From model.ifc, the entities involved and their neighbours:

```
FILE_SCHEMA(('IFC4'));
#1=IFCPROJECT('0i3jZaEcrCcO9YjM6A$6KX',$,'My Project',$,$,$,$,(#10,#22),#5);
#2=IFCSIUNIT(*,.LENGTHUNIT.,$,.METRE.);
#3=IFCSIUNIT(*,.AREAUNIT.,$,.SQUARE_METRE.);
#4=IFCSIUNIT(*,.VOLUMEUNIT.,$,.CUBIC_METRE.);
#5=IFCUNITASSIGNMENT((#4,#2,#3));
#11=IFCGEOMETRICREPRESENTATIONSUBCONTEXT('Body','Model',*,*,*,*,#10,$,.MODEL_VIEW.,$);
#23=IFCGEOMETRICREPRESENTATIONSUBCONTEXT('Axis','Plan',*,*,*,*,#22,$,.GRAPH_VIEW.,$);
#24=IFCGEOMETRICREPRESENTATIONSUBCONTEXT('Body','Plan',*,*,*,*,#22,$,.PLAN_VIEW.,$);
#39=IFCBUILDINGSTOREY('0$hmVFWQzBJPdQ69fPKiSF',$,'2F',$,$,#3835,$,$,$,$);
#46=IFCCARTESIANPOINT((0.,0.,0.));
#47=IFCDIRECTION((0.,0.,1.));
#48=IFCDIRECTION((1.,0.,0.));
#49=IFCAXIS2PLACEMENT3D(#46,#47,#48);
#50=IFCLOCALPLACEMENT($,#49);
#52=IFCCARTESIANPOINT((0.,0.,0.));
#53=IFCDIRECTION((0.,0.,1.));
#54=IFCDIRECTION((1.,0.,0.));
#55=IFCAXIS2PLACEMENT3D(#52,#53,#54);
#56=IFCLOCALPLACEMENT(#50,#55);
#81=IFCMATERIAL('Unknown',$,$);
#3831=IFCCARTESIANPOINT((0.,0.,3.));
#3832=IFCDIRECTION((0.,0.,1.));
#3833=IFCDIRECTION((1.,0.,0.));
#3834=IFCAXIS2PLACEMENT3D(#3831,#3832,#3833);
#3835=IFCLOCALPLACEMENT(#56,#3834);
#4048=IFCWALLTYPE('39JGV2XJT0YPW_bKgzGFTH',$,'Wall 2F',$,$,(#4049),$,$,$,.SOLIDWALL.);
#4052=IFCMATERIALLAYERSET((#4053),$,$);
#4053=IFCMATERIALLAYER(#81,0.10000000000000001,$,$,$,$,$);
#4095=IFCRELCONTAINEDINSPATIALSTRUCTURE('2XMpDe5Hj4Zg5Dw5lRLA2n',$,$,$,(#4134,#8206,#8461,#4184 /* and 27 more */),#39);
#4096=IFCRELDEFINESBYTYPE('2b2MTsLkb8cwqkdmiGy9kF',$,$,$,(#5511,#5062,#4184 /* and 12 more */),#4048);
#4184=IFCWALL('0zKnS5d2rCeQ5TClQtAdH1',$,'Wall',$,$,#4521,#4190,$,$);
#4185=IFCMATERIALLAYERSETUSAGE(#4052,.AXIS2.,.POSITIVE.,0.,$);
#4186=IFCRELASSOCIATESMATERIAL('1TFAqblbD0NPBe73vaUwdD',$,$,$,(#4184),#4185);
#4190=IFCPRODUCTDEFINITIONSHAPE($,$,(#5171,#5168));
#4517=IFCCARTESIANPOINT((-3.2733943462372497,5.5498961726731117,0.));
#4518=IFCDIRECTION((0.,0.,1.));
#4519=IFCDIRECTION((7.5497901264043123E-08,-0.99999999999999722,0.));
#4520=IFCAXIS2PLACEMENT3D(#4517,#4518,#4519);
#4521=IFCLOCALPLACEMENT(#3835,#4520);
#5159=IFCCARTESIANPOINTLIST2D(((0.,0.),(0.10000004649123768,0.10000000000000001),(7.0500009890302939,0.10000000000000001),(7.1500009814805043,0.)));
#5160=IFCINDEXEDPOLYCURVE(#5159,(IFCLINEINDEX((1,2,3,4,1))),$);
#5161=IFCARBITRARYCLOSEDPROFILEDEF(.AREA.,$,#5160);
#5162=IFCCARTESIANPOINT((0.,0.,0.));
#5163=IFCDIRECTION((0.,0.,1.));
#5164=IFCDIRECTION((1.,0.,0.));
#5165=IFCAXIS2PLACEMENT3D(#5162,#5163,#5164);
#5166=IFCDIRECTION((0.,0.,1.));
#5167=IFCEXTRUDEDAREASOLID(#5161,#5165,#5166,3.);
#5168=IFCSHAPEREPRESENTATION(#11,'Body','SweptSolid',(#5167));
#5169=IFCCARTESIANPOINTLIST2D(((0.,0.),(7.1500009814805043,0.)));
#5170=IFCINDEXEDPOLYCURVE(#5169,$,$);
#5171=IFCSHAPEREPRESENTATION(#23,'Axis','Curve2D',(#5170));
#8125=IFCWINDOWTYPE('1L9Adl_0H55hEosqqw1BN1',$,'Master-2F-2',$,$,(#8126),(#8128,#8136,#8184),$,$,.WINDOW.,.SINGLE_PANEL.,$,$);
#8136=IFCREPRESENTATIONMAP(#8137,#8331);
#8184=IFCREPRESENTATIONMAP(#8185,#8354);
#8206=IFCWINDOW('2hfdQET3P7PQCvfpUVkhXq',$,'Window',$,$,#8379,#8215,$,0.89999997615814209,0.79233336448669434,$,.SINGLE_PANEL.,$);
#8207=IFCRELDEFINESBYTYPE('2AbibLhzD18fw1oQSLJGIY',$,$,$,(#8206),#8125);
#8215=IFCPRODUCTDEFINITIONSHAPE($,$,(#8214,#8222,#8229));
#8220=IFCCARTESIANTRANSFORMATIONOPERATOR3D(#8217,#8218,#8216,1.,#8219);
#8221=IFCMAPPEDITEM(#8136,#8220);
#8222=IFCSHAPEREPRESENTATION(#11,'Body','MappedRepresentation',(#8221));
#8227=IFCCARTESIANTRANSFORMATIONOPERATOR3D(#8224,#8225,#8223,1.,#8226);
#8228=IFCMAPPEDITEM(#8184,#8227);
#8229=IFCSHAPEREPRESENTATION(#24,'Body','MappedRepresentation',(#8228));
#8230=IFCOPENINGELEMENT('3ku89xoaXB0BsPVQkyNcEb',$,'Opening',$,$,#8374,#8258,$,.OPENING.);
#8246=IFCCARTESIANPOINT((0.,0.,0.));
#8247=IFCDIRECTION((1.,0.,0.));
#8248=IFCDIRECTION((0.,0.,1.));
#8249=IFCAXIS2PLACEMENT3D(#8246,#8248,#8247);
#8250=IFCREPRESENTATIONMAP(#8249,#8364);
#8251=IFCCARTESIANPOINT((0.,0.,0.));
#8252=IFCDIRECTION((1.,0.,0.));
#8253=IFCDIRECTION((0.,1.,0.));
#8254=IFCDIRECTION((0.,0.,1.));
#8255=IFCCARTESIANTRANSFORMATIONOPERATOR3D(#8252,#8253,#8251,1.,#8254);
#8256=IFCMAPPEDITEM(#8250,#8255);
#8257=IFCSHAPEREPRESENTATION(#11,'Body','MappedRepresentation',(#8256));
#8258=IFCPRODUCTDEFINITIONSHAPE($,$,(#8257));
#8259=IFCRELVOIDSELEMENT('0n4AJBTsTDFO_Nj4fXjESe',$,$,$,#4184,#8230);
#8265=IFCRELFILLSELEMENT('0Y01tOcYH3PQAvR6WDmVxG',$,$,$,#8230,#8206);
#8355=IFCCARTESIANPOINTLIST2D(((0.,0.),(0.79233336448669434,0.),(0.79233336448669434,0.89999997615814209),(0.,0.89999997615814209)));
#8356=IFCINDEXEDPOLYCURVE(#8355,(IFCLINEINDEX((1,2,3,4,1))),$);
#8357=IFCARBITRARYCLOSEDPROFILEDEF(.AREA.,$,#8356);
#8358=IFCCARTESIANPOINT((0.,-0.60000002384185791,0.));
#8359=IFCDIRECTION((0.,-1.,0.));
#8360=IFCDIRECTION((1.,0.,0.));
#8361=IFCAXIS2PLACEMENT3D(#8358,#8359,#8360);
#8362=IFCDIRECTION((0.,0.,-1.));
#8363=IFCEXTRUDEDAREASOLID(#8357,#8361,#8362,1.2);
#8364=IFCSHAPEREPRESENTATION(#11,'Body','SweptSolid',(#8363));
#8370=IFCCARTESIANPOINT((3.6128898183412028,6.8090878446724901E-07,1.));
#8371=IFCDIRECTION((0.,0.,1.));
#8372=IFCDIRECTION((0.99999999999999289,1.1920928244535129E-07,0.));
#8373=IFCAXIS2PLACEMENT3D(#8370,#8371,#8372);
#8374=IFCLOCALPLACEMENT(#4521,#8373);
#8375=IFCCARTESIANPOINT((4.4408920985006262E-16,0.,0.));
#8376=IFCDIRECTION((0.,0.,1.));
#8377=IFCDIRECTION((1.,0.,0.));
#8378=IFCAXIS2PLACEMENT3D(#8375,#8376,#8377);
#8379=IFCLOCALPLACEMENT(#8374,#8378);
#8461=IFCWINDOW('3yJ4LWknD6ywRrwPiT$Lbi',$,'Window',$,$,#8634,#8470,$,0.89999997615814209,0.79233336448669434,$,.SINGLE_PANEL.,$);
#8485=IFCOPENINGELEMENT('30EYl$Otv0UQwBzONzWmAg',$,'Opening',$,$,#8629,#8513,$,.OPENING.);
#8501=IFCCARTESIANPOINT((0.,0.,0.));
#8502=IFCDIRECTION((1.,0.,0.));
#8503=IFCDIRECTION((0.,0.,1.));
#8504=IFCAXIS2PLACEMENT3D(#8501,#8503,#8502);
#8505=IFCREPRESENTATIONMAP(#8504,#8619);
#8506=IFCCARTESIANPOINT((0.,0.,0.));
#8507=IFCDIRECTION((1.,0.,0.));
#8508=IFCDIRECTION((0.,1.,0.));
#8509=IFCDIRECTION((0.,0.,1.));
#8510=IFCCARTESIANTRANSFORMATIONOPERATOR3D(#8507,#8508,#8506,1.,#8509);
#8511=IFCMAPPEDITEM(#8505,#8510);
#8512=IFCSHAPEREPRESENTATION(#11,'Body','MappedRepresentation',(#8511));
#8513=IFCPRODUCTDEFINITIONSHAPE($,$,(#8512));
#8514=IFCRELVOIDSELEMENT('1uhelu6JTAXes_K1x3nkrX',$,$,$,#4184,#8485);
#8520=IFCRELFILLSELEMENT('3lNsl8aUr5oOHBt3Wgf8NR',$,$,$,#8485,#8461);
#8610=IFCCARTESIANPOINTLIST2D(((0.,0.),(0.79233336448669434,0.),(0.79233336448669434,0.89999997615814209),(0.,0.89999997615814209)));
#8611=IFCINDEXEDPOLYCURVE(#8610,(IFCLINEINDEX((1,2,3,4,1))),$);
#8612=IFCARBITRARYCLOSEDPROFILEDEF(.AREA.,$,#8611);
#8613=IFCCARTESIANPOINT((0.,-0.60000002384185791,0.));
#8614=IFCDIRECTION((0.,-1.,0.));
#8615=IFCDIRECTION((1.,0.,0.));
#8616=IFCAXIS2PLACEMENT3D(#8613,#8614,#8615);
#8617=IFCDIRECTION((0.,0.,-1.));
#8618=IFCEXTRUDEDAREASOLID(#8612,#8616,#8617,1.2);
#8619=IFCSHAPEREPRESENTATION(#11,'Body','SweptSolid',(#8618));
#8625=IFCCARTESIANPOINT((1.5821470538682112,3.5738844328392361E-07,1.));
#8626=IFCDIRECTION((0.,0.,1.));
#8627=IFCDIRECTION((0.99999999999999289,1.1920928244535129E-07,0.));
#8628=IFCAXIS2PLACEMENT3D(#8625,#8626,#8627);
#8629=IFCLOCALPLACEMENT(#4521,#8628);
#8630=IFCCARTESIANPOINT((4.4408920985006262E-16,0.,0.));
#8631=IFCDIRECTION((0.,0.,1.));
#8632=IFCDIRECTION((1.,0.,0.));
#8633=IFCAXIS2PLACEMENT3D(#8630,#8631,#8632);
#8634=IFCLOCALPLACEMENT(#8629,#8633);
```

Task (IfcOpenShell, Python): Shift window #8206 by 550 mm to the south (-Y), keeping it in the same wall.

```python
import ifcopenshell
import ifcopenshell.api.geometry
import ifcopenshell.util.placement
import ifcopenshell.util.unit

model = ifcopenshell.open("model.ifc")
unit_scale = ifcopenshell.util.unit.calculate_unit_scale(model)

window = model.by_guid("2hfdQET3P7PQCvfpUVkhXq")
opening = window.FillsVoids[0].RelatingOpeningElement
wall = opening.VoidsElements[0].RelatingBuildingElement

wall_matrix = ifcopenshell.util.placement.get_local_placement(wall.ObjectPlacement)
shift = wall_matrix[:3, 0] * 0.55 / unit_scale
before = ifcopenshell.util.placement.get_local_placement(window.ObjectPlacement)[:3, 3].copy()

# The window is placed relative to its opening, so it follows when the opening moves.
matrix = ifcopenshell.util.placement.get_local_placement(opening.ObjectPlacement)
matrix[:3, 3] += shift
ifcopenshell.api.geometry.edit_object_placement(
    model, product=opening, matrix=matrix, is_si=False, should_transform_children=True
)

after = ifcopenshell.util.placement.get_local_placement(window.ObjectPlacement)[:3, 3]
print("window moved by", (after - before).round(3) + 0.0)

model.write("model_rev.ifc")
```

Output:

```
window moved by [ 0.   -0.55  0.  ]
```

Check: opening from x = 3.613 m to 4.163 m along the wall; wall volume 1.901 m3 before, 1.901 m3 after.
